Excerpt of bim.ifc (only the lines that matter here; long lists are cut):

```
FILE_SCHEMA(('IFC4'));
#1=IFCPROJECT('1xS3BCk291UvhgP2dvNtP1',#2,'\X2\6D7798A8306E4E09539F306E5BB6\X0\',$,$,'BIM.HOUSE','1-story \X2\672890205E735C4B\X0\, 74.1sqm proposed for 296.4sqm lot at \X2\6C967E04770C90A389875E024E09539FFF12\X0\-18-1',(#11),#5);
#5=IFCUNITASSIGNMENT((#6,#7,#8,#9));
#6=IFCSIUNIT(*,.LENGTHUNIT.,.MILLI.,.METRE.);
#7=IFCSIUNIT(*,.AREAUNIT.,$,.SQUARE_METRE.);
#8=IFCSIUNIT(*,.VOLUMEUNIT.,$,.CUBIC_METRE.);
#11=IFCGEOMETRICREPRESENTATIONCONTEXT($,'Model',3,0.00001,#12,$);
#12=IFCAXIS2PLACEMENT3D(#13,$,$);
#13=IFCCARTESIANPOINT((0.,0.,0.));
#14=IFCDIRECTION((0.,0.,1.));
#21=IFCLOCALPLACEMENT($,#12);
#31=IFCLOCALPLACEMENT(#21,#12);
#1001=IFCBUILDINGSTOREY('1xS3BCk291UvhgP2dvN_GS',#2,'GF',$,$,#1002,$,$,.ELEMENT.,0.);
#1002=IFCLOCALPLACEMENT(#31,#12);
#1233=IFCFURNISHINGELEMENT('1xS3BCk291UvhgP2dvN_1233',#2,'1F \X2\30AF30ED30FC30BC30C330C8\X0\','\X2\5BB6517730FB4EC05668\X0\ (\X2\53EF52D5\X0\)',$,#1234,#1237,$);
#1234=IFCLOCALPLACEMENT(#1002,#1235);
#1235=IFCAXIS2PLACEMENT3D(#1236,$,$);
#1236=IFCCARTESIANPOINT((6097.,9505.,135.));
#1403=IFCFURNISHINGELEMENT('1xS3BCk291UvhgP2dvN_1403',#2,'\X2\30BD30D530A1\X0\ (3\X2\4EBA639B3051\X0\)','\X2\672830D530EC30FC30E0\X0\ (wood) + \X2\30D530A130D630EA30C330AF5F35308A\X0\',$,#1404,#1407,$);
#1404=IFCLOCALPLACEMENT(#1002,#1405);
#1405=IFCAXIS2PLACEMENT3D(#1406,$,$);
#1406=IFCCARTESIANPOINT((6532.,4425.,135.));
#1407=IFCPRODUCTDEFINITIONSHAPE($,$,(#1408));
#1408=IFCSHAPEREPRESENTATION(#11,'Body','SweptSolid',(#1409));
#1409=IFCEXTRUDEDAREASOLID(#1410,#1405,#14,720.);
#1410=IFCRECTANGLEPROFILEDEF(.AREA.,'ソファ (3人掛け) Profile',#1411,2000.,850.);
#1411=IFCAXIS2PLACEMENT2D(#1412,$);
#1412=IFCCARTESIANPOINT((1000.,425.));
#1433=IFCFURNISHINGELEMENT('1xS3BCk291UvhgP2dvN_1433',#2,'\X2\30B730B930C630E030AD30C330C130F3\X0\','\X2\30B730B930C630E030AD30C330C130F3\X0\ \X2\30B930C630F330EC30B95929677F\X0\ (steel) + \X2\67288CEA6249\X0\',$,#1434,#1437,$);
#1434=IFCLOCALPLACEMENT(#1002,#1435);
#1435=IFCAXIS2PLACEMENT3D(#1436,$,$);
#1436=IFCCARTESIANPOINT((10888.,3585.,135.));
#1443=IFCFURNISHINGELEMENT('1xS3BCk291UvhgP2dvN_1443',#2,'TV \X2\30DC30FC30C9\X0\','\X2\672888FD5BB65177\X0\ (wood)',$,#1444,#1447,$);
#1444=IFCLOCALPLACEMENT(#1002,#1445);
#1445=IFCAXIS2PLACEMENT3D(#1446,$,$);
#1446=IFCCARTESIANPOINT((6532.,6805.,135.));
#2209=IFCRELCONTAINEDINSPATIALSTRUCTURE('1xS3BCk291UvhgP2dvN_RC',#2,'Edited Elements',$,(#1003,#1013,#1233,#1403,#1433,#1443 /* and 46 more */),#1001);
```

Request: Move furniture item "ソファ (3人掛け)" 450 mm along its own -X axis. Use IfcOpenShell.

```python
import ifcopenshell
import ifcopenshell.api.geometry
import ifcopenshell.util.placement
import ifcopenshell.util.unit

model = ifcopenshell.open("bim.ifc")
unit_scale = ifcopenshell.util.unit.calculate_unit_scale(model)

item = model.by_guid("1xS3BCk291UvhgP2dvN_1403")
matrix = ifcopenshell.util.placement.get_local_placement(item.ObjectPlacement)
matrix[:3, 3] -= matrix[:3, 0] * 0.45 / unit_scale
ifcopenshell.api.geometry.edit_object_placement(model, product=item, matrix=matrix, is_si=False)

print(ifcopenshell.util.placement.get_local_placement(item.ObjectPlacement).round(3) + 0.0)

model.write("bim_v2.ifc")
```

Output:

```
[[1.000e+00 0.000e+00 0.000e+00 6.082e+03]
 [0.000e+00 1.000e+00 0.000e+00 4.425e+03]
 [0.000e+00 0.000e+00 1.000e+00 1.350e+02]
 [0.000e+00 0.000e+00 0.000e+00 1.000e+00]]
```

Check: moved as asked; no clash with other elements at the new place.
